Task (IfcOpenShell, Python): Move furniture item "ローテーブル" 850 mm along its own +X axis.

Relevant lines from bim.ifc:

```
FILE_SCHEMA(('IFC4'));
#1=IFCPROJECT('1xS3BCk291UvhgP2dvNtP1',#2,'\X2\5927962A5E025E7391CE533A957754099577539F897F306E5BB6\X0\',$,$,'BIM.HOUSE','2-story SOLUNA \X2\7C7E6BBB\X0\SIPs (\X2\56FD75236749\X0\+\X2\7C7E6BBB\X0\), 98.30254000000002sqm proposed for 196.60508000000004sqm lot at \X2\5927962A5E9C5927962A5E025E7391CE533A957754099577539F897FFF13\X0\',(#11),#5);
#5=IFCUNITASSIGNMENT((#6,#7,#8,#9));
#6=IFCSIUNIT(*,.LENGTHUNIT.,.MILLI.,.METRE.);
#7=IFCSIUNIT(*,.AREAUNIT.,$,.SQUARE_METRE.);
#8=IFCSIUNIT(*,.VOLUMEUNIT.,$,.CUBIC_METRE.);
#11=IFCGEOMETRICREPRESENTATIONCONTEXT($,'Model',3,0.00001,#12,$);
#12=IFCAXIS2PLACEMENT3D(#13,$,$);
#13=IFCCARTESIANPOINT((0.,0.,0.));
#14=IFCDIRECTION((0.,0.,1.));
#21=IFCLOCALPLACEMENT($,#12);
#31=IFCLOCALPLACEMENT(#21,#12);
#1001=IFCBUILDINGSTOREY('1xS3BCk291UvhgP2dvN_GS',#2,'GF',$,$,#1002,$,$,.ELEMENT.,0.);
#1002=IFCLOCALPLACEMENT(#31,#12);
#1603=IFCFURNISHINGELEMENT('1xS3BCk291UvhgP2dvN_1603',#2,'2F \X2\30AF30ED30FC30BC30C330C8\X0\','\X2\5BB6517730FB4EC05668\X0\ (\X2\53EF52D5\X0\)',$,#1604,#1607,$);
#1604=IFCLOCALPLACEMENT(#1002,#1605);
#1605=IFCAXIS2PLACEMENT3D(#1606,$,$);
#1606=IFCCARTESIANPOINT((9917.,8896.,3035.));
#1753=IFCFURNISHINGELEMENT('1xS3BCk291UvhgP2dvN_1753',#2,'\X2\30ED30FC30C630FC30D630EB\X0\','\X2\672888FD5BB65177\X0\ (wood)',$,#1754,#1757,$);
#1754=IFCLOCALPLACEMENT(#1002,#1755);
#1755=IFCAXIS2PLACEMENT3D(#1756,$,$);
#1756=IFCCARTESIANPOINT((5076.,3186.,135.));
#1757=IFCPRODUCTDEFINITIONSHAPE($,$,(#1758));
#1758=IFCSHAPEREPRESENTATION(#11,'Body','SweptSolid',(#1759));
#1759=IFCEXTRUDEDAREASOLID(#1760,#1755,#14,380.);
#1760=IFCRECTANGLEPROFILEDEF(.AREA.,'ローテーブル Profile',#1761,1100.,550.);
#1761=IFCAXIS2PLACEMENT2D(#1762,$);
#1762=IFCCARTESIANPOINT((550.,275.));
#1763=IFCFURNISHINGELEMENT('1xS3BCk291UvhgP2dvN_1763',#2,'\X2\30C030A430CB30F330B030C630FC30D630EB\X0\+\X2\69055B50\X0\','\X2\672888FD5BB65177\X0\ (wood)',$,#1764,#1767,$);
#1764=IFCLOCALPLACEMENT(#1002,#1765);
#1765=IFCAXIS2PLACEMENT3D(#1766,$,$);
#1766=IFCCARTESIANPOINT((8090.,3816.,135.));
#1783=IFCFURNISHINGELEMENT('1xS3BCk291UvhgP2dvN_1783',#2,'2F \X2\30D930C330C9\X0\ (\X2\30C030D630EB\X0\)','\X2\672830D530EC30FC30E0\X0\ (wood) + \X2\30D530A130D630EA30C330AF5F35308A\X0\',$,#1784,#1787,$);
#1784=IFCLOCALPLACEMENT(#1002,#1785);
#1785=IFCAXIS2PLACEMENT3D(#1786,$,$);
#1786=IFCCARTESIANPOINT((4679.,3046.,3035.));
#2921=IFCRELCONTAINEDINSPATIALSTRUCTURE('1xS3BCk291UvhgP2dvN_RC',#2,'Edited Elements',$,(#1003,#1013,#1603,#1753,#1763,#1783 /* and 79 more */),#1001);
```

```python
import ifcopenshell
import ifcopenshell.api.geometry
import ifcopenshell.util.placement

model = ifcopenshell.open("bim.ifc")

item = model.by_guid("1xS3BCk291UvhgP2dvN_1753")
matrix = ifcopenshell.util.placement.get_local_placement(item.ObjectPlacement)
matrix[:3, 3] += matrix[:3, 0] * 850.0
ifcopenshell.api.geometry.edit_object_placement(model, product=item, matrix=matrix, is_si=False)

print(ifcopenshell.util.placement.get_local_placement(item.ObjectPlacement).round(3) + 0.0)

model.write("bim_rev.ifc")
```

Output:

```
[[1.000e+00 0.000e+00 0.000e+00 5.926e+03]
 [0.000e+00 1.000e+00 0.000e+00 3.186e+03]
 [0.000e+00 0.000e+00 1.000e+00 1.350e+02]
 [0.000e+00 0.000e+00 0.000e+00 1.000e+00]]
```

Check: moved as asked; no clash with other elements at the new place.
